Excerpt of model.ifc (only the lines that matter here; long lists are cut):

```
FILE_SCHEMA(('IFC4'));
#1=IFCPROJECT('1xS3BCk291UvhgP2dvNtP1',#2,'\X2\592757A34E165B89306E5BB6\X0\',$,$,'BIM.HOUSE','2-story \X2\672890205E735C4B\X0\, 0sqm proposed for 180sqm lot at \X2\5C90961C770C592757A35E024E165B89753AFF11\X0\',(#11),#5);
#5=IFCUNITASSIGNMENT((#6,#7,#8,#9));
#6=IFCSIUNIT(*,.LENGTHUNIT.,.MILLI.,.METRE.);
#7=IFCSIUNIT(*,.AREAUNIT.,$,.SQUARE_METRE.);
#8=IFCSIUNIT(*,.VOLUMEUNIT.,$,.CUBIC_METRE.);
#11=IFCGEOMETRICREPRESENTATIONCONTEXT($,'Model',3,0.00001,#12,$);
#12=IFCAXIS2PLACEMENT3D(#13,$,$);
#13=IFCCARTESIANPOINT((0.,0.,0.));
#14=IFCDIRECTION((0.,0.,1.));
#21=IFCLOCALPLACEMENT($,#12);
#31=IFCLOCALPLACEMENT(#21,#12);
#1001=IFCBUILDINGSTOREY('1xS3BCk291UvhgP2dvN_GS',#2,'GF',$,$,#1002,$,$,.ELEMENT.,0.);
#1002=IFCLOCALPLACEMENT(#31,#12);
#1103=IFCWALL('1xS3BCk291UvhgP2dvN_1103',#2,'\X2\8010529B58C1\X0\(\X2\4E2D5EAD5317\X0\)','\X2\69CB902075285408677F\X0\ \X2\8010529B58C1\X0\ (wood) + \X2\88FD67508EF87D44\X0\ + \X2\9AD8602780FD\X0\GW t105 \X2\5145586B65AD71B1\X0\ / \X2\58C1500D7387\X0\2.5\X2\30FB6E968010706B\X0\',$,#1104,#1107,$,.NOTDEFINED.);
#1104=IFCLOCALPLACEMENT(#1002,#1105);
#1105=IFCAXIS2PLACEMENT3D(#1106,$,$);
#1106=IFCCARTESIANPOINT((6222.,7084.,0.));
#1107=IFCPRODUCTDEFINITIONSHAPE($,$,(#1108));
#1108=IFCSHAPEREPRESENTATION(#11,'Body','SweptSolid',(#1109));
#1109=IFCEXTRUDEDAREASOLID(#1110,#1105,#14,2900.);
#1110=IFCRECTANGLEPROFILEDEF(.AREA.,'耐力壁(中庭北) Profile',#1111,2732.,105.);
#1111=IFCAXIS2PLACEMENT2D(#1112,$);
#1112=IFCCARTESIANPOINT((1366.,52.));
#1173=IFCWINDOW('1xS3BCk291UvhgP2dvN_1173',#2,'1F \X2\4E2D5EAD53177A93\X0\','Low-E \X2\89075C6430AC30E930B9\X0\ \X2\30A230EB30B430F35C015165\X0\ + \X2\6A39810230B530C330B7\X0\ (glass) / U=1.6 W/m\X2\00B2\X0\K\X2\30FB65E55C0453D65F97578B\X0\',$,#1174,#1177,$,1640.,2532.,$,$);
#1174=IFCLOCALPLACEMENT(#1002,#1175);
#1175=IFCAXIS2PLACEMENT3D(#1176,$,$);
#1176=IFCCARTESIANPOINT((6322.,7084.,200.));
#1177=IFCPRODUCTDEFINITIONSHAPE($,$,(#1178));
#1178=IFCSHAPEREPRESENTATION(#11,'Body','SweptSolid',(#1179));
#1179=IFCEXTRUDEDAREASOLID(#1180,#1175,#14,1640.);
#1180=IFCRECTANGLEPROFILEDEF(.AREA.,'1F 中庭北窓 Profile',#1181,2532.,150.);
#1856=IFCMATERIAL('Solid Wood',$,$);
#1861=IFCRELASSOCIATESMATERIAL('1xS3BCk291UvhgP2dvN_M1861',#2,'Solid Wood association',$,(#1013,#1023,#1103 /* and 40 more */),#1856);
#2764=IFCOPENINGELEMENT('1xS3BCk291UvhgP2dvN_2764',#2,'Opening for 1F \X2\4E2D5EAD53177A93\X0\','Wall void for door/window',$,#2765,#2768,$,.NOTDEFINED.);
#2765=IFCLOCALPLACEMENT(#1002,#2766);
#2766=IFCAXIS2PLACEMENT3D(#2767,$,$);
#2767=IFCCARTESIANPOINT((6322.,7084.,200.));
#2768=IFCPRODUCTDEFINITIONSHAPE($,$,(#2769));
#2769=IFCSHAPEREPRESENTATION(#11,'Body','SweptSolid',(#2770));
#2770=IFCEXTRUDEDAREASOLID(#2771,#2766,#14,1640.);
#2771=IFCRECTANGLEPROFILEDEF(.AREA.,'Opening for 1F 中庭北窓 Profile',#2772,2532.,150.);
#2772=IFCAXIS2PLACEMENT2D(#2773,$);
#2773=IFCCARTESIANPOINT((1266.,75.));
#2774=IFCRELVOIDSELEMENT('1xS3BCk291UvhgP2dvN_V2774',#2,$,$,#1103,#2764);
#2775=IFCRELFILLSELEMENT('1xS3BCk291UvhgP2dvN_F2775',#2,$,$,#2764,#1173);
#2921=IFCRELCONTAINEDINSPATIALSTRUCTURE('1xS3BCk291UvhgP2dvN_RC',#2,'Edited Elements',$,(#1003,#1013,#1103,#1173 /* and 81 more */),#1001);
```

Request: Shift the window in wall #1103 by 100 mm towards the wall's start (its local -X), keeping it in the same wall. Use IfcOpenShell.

```python
import ifcopenshell
import ifcopenshell.api.geometry
import ifcopenshell.util.placement
import ifcopenshell.util.unit

model = ifcopenshell.open("model.ifc")
unit_scale = ifcopenshell.util.unit.calculate_unit_scale(model)

window = model.by_id(1173)
opening = window.FillsVoids[0].RelatingOpeningElement
wall = opening.VoidsElements[0].RelatingBuildingElement

wall_matrix = ifcopenshell.util.placement.get_local_placement(wall.ObjectPlacement)
shift = wall_matrix[:3, 0] * -0.1 / unit_scale
before = ifcopenshell.util.placement.get_local_placement(window.ObjectPlacement)[:3, 3].copy()

# The window is not placed relative to its opening, so move both.
for product in (opening, window):
    matrix = ifcopenshell.util.placement.get_local_placement(product.ObjectPlacement)
    matrix[:3, 3] += shift
    ifcopenshell.api.geometry.edit_object_placement(model, product=product, matrix=matrix, is_si=False)

after = ifcopenshell.util.placement.get_local_placement(window.ObjectPlacement)[:3, 3]
print("window moved by", (after - before).round(3) + 0.0)

model.write("model_updated.ifc")
```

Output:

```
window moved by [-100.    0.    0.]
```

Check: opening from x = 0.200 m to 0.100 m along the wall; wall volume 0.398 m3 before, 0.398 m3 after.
